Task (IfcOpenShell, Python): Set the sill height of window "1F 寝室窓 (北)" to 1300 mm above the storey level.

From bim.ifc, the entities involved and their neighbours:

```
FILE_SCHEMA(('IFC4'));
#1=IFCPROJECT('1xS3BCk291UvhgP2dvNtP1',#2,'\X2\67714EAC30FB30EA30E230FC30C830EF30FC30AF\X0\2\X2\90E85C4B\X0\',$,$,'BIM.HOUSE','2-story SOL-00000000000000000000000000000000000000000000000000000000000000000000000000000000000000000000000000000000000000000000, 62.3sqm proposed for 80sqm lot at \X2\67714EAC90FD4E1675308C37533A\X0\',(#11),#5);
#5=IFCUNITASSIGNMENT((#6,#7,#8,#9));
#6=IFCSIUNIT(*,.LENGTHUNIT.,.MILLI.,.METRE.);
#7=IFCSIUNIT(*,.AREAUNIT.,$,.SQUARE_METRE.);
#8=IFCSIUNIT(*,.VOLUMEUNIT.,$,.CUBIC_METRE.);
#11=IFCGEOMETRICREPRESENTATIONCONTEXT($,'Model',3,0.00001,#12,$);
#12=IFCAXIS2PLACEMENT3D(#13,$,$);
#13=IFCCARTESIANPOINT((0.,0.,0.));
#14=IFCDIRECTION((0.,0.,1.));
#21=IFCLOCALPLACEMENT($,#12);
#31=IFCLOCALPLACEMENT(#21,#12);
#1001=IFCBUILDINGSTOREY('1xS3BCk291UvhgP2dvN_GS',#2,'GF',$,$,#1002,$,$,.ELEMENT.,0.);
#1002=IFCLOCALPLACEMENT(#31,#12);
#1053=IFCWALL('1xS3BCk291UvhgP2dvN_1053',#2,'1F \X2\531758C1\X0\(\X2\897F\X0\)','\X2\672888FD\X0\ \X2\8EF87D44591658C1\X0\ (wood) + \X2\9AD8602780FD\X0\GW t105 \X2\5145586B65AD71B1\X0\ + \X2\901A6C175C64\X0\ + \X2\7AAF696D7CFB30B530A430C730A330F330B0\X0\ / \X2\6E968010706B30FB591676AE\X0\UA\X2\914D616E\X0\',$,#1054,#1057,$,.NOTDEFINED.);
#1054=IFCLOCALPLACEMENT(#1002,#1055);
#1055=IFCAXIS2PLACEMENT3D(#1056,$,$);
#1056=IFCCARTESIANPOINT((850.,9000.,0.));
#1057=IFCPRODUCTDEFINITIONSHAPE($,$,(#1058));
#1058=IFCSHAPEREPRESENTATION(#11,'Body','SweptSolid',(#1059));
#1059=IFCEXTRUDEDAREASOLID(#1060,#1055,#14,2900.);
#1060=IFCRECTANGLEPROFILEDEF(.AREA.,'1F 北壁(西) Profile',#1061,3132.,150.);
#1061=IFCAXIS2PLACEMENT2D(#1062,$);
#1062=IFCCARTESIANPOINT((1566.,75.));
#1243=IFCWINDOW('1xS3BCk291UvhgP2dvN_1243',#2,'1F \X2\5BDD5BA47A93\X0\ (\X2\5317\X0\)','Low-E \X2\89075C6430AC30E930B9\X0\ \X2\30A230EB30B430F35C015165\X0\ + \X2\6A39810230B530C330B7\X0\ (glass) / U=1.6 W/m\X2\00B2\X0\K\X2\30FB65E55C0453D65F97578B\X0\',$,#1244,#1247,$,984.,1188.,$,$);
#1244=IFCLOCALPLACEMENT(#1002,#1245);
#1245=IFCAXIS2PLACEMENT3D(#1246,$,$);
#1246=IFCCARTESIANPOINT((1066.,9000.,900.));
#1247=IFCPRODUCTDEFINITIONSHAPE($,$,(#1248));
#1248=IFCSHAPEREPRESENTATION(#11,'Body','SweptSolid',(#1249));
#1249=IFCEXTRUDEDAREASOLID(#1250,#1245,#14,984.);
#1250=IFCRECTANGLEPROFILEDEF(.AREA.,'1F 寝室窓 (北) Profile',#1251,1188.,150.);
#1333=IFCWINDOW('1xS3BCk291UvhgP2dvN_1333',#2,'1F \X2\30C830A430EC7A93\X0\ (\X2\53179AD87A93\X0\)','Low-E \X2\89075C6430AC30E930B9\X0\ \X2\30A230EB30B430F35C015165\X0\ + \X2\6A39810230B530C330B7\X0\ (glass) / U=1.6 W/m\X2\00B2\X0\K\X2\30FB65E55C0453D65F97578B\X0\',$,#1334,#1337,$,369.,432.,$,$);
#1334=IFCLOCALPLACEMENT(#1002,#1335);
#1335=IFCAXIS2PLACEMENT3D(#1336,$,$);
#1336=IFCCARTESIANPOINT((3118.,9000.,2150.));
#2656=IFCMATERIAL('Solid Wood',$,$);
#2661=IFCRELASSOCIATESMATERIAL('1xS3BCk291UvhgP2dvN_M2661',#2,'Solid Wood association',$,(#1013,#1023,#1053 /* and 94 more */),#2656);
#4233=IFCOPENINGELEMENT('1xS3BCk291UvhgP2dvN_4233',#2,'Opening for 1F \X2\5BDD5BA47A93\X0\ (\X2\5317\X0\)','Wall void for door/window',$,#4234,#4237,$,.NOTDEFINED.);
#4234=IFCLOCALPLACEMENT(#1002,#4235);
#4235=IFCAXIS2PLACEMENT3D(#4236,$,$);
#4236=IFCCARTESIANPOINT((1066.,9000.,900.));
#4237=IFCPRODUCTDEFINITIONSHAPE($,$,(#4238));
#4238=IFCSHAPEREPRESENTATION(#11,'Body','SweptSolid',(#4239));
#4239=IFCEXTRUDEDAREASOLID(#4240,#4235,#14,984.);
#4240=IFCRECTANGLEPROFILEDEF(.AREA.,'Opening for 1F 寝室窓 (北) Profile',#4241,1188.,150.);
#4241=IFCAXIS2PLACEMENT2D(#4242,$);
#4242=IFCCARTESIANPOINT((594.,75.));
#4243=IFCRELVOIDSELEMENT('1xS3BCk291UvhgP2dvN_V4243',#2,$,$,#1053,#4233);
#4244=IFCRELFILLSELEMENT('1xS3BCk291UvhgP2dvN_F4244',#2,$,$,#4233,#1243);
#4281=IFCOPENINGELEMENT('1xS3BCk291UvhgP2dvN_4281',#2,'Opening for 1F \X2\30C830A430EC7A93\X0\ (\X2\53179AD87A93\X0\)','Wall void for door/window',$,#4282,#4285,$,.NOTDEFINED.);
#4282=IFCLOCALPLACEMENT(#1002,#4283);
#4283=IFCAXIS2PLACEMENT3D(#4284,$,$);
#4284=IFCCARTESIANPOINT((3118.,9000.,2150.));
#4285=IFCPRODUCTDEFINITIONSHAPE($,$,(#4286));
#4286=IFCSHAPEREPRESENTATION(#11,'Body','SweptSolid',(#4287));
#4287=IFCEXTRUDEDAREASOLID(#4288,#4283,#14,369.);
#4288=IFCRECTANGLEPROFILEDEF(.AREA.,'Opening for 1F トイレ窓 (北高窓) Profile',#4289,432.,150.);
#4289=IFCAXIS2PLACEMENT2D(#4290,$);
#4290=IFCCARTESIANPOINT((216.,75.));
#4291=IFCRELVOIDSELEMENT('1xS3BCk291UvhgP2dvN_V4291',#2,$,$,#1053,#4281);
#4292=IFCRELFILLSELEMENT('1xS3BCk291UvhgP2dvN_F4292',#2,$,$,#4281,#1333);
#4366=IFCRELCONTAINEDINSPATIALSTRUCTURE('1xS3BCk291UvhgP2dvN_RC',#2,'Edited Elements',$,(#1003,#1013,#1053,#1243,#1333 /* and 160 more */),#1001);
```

```python
import numpy as np
import ifcopenshell
import ifcopenshell.api.geometry
import ifcopenshell.geom
import ifcopenshell.util.element
import ifcopenshell.util.placement
import ifcopenshell.util.shape
import ifcopenshell.util.unit

model = ifcopenshell.open("bim.ifc")
unit_scale = ifcopenshell.util.unit.calculate_unit_scale(model)

window = model.by_id(1243)
opening = window.FillsVoids[0].RelatingOpeningElement
storey = ifcopenshell.util.element.get_container(window, ifc_class="IfcBuildingStorey")
level = ifcopenshell.util.placement.get_local_placement(storey.ObjectPlacement)[2, 3]

# The opening's origin need not be at the sill, so measure its lowest point.
shape = ifcopenshell.geom.create_shape(ifcopenshell.geom.settings(), opening)
bottom = ifcopenshell.util.shape.get_shape_bottom_elevation(shape, shape.geometry) / unit_scale
dz = level + 1300.0 - bottom

shift = np.array([0.0, 0.0, dz])
# The window is not placed relative to its opening, so move both.
for product in (opening, window):
    matrix = ifcopenshell.util.placement.get_local_placement(product.ObjectPlacement)
    matrix[:3, 3] += shift
    ifcopenshell.api.geometry.edit_object_placement(model, product=product, matrix=matrix, is_si=False)

print(f"moved by {dz * unit_scale:+.3f} m")

model.write("bim_v2.ifc")
```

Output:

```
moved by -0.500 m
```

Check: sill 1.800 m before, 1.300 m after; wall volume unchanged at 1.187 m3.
